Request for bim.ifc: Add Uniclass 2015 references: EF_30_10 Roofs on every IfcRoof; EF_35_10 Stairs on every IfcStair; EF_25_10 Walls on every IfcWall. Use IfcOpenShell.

First a look at what the model holds.

```python
import ifcopenshell

model = ifcopenshell.open("bim.ifc")
print(model.schema)
print("classifications:", [c.Name for c in model.by_type("IfcClassification")])
for ifc_class in ("IfcDoor", "IfcRoof", "IfcStair", "IfcWall", "IfcWindow"):
    print(ifc_class, len(model.by_type(ifc_class)))
```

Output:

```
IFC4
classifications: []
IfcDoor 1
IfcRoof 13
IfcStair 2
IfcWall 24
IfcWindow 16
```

```python
import ifcopenshell
import ifcopenshell.api.classification

model = ifcopenshell.open("bim.ifc")

system = ifcopenshell.api.classification.add_classification(model, classification="Uniclass 2015")

codes = {
    "IfcRoof": ("EF_30_10", "Roofs"),
    "IfcStair": ("EF_35_10", "Stairs"),
    "IfcWall": ("EF_25_10", "Walls"),
}
for ifc_class, (code, name) in codes.items():
    products = model.by_type(ifc_class)
    ifcopenshell.api.classification.add_reference(
        model, products=products, classification=system, identification=code, name=name
    )
    print(code, len(products))

model.write("bim_edited.ifc")
```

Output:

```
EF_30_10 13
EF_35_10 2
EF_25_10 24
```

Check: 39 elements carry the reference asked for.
